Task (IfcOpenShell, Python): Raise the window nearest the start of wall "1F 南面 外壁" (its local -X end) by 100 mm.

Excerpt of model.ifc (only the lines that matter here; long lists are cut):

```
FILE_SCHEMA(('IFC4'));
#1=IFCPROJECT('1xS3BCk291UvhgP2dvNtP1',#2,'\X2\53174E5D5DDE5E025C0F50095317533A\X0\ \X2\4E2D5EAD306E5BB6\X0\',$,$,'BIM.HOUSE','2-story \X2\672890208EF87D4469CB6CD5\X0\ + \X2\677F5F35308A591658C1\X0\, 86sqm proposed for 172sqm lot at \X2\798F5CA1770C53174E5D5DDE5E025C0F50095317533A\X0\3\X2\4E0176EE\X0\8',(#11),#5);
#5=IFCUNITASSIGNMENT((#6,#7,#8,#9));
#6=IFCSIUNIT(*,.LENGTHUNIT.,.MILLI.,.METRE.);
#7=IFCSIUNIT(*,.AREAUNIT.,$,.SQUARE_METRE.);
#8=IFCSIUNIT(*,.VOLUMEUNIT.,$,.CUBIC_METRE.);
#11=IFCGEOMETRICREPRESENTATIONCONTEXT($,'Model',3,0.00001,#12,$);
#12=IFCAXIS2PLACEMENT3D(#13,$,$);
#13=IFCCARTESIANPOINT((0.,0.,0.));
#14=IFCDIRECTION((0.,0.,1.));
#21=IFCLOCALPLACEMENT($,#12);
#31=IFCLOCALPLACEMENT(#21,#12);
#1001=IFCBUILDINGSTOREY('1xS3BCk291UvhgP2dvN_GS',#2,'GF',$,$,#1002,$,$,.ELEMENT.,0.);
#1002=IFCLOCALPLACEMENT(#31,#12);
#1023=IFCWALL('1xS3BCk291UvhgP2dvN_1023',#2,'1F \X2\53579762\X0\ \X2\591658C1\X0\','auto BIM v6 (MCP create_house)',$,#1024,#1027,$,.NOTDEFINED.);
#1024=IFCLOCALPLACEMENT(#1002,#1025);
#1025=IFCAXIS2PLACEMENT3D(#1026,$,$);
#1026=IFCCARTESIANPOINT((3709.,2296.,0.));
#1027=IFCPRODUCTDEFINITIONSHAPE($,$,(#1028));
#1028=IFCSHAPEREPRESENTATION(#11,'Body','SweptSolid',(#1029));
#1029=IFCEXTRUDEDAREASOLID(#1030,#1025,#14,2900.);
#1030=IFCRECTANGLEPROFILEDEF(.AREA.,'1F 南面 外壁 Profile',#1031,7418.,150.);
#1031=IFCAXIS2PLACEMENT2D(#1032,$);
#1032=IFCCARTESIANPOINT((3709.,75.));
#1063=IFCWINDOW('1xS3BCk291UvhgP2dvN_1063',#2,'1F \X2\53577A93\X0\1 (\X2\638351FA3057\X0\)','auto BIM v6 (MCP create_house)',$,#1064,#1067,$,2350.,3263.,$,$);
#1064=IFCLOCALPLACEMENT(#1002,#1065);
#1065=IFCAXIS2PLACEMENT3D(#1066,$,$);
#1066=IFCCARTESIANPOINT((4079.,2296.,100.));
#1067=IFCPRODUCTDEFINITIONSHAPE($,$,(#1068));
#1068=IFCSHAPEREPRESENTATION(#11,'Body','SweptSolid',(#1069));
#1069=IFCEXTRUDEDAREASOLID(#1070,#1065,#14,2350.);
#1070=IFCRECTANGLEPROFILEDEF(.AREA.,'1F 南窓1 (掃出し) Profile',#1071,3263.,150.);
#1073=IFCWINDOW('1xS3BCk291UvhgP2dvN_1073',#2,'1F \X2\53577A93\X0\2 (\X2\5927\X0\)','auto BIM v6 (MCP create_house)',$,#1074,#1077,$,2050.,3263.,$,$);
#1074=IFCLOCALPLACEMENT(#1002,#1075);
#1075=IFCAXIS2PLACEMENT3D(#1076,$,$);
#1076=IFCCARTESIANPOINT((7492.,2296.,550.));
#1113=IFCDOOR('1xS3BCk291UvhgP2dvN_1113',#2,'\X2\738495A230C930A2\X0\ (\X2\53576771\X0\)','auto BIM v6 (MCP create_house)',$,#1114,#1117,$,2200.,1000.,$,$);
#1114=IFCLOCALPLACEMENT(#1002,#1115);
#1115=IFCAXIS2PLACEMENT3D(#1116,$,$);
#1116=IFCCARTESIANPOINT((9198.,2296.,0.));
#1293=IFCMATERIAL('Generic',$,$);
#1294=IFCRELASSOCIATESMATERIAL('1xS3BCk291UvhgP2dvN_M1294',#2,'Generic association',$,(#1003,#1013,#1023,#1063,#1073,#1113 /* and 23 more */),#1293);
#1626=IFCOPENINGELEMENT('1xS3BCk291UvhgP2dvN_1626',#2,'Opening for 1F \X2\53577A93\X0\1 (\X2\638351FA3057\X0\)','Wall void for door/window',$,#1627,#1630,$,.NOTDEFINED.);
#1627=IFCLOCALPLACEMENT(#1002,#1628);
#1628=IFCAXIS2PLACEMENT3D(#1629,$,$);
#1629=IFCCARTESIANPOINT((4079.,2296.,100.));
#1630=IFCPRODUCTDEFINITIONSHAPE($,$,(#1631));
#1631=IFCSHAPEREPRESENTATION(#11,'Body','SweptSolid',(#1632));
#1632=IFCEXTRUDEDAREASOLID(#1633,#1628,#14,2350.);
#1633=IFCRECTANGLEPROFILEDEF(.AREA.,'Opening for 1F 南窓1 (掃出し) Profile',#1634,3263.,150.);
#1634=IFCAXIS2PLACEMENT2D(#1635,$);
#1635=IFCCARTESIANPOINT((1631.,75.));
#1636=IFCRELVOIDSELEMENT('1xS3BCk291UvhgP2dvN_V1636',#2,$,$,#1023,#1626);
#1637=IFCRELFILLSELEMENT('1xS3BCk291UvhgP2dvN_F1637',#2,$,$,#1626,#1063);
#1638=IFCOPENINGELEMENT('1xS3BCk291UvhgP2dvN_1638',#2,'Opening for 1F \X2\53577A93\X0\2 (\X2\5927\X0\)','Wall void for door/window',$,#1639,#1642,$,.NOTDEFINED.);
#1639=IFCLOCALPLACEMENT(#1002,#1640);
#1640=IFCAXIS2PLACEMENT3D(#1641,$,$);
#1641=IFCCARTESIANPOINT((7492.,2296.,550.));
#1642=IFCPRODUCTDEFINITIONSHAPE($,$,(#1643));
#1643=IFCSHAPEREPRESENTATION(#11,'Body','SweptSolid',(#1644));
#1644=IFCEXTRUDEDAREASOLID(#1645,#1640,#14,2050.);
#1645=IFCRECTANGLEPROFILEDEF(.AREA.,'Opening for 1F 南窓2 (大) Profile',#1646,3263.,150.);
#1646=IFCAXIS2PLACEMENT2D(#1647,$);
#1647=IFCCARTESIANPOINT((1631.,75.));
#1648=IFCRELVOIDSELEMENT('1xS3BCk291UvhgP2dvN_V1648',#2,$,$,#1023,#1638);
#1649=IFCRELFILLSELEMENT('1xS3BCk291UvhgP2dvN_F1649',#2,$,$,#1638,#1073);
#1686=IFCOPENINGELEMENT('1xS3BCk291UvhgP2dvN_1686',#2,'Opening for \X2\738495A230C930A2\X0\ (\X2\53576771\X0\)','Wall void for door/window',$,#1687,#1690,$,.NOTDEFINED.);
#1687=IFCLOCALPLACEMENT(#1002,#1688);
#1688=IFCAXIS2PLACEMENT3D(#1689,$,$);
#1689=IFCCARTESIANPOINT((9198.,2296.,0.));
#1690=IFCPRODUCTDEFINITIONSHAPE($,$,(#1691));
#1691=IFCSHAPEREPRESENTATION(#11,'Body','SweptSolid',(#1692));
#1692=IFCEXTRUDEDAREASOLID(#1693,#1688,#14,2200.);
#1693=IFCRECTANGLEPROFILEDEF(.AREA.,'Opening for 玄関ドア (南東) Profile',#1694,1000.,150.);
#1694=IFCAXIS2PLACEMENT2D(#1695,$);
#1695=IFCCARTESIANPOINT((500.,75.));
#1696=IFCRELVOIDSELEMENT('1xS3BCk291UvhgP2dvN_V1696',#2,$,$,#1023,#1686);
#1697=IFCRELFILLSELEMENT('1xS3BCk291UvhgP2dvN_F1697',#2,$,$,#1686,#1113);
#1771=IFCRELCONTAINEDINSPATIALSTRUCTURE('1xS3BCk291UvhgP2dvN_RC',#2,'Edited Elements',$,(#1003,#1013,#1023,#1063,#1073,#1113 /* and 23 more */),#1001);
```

```python
import numpy as np
import ifcopenshell
import ifcopenshell.api.geometry
import ifcopenshell.util.placement
import ifcopenshell.util.unit

model = ifcopenshell.open("model.ifc")
unit_scale = ifcopenshell.util.unit.calculate_unit_scale(model)

window = model.by_guid("1xS3BCk291UvhgP2dvN_1063")
opening = window.FillsVoids[0].RelatingOpeningElement
dz = 0.1 / unit_scale

shift = np.array([0.0, 0.0, dz])
# The window is not placed relative to its opening, so move both.
for product in (opening, window):
    matrix = ifcopenshell.util.placement.get_local_placement(product.ObjectPlacement)
    matrix[:3, 3] += shift
    ifcopenshell.api.geometry.edit_object_placement(model, product=product, matrix=matrix, is_si=False)

print(f"moved by {dz * unit_scale:+.3f} m")

model.write("model_rev.ifc")
```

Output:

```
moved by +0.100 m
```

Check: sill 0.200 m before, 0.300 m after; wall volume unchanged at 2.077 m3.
